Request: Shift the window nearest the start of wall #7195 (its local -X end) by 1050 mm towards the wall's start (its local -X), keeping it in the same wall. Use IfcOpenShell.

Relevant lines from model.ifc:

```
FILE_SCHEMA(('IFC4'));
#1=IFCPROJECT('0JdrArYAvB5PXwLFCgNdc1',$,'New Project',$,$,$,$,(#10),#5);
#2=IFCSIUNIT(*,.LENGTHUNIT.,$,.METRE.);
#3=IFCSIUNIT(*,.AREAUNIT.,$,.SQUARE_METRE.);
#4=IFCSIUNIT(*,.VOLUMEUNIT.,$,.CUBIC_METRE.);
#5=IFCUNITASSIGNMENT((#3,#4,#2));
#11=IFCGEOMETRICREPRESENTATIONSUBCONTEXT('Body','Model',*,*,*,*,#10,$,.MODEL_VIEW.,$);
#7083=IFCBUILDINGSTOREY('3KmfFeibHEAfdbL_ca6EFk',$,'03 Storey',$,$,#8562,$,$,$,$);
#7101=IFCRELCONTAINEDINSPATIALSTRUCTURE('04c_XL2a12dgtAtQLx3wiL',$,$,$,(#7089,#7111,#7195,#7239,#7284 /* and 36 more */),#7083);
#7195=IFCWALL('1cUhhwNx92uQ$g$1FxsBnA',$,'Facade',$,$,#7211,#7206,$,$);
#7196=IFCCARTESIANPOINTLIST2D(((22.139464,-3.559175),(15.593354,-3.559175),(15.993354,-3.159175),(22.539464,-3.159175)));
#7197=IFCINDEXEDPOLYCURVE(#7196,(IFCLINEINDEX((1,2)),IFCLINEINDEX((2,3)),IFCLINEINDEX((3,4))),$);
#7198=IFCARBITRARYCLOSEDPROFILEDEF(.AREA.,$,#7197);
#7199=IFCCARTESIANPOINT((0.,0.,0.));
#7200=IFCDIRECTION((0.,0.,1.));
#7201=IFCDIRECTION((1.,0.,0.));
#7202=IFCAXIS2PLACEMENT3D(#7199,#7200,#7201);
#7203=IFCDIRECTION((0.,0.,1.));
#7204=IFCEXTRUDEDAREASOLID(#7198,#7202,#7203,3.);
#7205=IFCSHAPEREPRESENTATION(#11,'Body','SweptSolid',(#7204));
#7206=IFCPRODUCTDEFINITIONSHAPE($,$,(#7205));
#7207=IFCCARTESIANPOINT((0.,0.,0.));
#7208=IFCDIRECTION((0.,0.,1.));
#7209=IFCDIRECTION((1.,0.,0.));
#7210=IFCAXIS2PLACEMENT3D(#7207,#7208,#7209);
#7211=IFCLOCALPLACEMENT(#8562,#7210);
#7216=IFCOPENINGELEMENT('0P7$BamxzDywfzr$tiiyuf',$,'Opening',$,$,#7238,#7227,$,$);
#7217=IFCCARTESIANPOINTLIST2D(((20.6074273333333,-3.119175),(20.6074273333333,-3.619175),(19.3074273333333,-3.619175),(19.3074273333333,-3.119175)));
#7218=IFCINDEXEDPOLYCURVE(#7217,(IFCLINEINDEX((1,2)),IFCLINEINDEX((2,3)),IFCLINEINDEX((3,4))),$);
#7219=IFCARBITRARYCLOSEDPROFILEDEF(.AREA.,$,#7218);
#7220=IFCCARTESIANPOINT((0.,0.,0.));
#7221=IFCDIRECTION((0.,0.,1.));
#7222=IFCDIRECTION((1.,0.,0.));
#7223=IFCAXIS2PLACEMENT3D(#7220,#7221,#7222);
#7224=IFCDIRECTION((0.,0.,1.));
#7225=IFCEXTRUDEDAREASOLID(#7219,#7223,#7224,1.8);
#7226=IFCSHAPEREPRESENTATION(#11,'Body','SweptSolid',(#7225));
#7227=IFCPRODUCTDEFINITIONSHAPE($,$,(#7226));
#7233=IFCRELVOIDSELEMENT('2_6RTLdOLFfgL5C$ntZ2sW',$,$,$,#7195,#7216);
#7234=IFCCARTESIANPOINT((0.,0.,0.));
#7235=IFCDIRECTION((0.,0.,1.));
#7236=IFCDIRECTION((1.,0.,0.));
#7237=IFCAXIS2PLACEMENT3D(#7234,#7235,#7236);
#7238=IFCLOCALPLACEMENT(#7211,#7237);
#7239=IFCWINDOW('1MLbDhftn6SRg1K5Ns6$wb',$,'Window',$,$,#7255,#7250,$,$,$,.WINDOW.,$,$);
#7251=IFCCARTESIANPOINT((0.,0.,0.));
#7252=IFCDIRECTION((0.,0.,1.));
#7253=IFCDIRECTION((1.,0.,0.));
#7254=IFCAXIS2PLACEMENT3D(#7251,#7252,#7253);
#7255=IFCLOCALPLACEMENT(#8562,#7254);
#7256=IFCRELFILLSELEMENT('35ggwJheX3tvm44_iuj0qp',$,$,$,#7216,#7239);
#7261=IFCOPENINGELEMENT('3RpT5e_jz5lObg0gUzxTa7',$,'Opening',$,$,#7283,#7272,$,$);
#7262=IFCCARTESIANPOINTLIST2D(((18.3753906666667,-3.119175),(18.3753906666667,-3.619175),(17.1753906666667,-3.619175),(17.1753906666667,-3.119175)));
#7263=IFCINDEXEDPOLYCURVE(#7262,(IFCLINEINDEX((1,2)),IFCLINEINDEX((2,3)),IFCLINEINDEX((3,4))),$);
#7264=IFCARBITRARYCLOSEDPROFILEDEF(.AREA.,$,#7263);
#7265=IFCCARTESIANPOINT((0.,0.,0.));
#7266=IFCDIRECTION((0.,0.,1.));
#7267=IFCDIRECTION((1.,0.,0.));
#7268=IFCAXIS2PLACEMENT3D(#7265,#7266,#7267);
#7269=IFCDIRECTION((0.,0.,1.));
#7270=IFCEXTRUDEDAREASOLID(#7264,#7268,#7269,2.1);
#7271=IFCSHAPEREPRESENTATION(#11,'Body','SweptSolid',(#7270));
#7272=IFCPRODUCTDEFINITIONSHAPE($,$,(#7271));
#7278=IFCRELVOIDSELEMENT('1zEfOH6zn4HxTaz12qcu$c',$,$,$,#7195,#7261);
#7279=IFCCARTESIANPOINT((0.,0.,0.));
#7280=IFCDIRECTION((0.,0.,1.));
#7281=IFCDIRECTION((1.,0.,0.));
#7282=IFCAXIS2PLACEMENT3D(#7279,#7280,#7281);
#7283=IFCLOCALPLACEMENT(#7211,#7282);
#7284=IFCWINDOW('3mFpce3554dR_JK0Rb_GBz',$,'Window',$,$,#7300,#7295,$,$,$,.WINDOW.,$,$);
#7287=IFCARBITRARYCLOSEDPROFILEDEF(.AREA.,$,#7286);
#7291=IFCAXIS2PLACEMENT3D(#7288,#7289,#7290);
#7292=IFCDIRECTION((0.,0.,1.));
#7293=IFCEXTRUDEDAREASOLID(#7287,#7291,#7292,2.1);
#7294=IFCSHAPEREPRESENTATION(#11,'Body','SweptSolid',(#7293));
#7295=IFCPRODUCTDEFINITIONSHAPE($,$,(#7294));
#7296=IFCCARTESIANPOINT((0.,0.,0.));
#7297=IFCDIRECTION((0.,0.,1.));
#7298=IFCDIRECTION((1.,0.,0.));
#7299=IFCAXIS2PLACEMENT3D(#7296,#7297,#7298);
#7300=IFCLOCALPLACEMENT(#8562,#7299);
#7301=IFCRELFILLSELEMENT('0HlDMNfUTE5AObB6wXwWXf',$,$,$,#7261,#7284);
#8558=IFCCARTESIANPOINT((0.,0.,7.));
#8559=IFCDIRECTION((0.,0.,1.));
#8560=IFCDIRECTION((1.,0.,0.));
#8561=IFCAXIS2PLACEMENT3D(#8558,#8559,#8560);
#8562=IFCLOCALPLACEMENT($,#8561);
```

```python
import ifcopenshell
import ifcopenshell.api.geometry
import ifcopenshell.util.placement
import ifcopenshell.util.unit

model = ifcopenshell.open("model.ifc")
unit_scale = ifcopenshell.util.unit.calculate_unit_scale(model)

window = model.by_guid("3mFpce3554dR_JK0Rb_GBz")
opening = window.FillsVoids[0].RelatingOpeningElement
wall = opening.VoidsElements[0].RelatingBuildingElement

wall_matrix = ifcopenshell.util.placement.get_local_placement(wall.ObjectPlacement)
shift = wall_matrix[:3, 0] * -1.05 / unit_scale
before = ifcopenshell.util.placement.get_local_placement(window.ObjectPlacement)[:3, 3].copy()

# The window is not placed relative to its opening, so move both.
for product in (opening, window):
    matrix = ifcopenshell.util.placement.get_local_placement(product.ObjectPlacement)
    matrix[:3, 3] += shift
    ifcopenshell.api.geometry.edit_object_placement(model, product=product, matrix=matrix, is_si=False)

after = ifcopenshell.util.placement.get_local_placement(window.ObjectPlacement)[:3, 3]
print("window moved by", (after - before).round(3) + 0.0)

model.write("model_v2.ifc")
```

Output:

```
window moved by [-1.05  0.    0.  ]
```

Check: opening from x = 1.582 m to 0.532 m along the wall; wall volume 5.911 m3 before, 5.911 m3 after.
